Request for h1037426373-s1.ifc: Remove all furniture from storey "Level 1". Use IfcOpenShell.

First a look at what the model holds.

```python
import ifcopenshell
import ifcopenshell.util.element

model = ifcopenshell.open("h1037426373-s1.ifc")
print(model.schema)
storey = next(s for s in model.by_type("IfcBuildingStorey") if s.Name == "Level 1")
furniture = [e for e in ifcopenshell.util.element.get_decomposition(storey) if e.is_a("IfcFurnishingElement")]
seen = {}
for e in furniture:
    element_type = ifcopenshell.util.element.get_type(e)
    name = element_type.Name if element_type not in (None, e) else None
    seen[name] = seen.get(name, 0) + 1
for name, count in sorted(seen.items(), key=str):
    print(count, "x", name)
```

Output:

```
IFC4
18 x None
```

```python
import ifcopenshell
import ifcopenshell.api.root
import ifcopenshell.util.element

model = ifcopenshell.open("h1037426373-s1.ifc")

storey = next(s for s in model.by_type("IfcBuildingStorey") if s.Name == "Level 1")
furniture = [e for e in ifcopenshell.util.element.get_decomposition(storey) if e.is_a("IfcFurnishingElement")]

for e in furniture:
    ifcopenshell.api.root.remove_product(model, product=e)
print(len(furniture), "removed")

model.write("h1037426373-s1_updated.ifc")
```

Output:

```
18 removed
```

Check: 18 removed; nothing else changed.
